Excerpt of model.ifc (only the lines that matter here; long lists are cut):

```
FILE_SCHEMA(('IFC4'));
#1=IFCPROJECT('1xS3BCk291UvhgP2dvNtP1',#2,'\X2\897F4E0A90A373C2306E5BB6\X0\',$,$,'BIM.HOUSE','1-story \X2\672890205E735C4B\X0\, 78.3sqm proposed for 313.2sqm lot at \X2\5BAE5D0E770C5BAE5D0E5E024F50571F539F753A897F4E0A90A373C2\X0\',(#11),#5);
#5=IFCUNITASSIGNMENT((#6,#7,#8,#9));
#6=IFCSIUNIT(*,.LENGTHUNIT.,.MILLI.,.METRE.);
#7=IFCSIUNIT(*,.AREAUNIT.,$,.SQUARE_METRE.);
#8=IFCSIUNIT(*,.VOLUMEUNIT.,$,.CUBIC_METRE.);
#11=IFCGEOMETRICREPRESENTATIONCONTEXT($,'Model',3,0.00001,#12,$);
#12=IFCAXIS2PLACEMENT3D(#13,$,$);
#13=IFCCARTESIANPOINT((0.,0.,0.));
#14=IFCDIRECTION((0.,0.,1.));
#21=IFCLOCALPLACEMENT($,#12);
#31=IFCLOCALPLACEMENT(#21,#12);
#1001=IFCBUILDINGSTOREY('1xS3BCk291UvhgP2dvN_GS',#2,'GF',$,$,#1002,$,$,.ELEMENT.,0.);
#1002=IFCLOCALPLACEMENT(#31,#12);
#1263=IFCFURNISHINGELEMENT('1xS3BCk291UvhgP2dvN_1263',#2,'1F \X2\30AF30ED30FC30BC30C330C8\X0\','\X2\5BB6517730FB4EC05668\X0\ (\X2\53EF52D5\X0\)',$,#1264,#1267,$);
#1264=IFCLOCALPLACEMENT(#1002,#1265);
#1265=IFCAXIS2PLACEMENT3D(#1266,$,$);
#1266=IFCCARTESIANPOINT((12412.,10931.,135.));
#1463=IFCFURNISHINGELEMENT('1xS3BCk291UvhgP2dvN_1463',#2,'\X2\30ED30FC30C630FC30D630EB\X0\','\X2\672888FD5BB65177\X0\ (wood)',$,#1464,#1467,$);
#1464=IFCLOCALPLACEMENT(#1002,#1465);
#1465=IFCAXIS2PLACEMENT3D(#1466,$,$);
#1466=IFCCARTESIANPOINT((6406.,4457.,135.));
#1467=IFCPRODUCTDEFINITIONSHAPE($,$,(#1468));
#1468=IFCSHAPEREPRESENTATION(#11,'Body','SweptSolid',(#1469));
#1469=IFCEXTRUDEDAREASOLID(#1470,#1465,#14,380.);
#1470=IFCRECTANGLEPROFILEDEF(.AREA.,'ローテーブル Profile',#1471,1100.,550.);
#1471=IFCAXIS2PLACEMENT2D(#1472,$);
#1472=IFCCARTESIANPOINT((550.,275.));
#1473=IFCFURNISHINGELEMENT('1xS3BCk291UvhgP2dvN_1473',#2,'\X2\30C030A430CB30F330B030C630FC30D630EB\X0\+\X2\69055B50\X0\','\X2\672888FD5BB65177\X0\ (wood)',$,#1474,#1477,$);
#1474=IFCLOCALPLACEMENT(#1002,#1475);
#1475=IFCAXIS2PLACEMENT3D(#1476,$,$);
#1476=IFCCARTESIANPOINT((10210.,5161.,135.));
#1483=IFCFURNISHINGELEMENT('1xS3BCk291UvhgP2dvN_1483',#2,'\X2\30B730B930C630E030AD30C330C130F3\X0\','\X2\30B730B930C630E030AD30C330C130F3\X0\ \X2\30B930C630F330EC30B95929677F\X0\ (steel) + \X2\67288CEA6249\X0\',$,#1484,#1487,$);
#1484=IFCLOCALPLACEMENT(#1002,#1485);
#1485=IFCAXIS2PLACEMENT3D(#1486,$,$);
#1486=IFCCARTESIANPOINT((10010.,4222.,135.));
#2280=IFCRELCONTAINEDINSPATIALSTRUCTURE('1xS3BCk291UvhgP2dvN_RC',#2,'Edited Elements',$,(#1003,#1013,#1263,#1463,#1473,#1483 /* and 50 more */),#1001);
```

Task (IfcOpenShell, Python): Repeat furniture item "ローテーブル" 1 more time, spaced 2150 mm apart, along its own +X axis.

```python
import ifcopenshell
import ifcopenshell.api.geometry
import ifcopenshell.api.root
import ifcopenshell.util.element
import ifcopenshell.util.placement
import ifcopenshell.util.unit

model = ifcopenshell.open("model.ifc")
unit_scale = ifcopenshell.util.unit.calculate_unit_scale(model)


def reuse_history(source, copy):
    """copy_class also copies each property set's owner history, people and application; keep the originals."""
    for rel in copy.IsDefinedBy:
        if rel.is_a("IfcRelDefinesByProperties") and (history := rel.RelatingPropertyDefinition.OwnerHistory):
            rel.RelatingPropertyDefinition.OwnerHistory = source.OwnerHistory
            ifcopenshell.util.element.remove_deep2(model, history)


source = model.by_guid("1xS3BCk291UvhgP2dvN_1463")
base = ifcopenshell.util.placement.get_local_placement(source.ObjectPlacement)
step = base[:3, 0] * 2.15 / unit_scale

for i in range(1, 2):
    copy = ifcopenshell.api.root.copy_class(model, product=source)
    copy.Representation = ifcopenshell.util.element.copy_deep(
        model, source.Representation, exclude=["IfcGeometricRepresentationContext", "IfcRepresentationMap"]
    )
    reuse_history(source, copy)
    matrix = base.copy()
    matrix[:3, 3] += i * step
    print("added at", matrix[:3, 3].round(3) + 0.0)
    ifcopenshell.api.geometry.edit_object_placement(model, product=copy, matrix=matrix, is_si=False)

model.write("model_updated.ifc")
```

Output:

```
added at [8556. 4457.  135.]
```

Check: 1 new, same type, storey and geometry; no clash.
